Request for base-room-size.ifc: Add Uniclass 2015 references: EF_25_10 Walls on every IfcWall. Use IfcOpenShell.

First a look at what the model holds.

```python
import ifcopenshell

model = ifcopenshell.open("base-room-size.ifc")
print(model.schema)
print("classifications:", [c.Name for c in model.by_type("IfcClassification")])
for ifc_class in ("IfcDoor", "IfcRoof", "IfcStair", "IfcWall", "IfcWindow"):
    print(ifc_class, len(model.by_type(ifc_class)))
```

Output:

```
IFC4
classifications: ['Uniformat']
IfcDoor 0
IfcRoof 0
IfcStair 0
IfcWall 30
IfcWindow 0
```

```python
import ifcopenshell
import ifcopenshell.api.classification

model = ifcopenshell.open("base-room-size.ifc")

system = ifcopenshell.api.classification.add_classification(model, classification="Uniclass 2015")

codes = {
    "IfcWall": ("EF_25_10", "Walls"),
}
for ifc_class, (code, name) in codes.items():
    products = model.by_type(ifc_class)
    ifcopenshell.api.classification.add_reference(
        model, products=products, classification=system, identification=code, name=name
    )
    print(code, len(products))

model.write("base-room-size_edited.ifc")
```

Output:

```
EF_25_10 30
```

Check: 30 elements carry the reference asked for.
